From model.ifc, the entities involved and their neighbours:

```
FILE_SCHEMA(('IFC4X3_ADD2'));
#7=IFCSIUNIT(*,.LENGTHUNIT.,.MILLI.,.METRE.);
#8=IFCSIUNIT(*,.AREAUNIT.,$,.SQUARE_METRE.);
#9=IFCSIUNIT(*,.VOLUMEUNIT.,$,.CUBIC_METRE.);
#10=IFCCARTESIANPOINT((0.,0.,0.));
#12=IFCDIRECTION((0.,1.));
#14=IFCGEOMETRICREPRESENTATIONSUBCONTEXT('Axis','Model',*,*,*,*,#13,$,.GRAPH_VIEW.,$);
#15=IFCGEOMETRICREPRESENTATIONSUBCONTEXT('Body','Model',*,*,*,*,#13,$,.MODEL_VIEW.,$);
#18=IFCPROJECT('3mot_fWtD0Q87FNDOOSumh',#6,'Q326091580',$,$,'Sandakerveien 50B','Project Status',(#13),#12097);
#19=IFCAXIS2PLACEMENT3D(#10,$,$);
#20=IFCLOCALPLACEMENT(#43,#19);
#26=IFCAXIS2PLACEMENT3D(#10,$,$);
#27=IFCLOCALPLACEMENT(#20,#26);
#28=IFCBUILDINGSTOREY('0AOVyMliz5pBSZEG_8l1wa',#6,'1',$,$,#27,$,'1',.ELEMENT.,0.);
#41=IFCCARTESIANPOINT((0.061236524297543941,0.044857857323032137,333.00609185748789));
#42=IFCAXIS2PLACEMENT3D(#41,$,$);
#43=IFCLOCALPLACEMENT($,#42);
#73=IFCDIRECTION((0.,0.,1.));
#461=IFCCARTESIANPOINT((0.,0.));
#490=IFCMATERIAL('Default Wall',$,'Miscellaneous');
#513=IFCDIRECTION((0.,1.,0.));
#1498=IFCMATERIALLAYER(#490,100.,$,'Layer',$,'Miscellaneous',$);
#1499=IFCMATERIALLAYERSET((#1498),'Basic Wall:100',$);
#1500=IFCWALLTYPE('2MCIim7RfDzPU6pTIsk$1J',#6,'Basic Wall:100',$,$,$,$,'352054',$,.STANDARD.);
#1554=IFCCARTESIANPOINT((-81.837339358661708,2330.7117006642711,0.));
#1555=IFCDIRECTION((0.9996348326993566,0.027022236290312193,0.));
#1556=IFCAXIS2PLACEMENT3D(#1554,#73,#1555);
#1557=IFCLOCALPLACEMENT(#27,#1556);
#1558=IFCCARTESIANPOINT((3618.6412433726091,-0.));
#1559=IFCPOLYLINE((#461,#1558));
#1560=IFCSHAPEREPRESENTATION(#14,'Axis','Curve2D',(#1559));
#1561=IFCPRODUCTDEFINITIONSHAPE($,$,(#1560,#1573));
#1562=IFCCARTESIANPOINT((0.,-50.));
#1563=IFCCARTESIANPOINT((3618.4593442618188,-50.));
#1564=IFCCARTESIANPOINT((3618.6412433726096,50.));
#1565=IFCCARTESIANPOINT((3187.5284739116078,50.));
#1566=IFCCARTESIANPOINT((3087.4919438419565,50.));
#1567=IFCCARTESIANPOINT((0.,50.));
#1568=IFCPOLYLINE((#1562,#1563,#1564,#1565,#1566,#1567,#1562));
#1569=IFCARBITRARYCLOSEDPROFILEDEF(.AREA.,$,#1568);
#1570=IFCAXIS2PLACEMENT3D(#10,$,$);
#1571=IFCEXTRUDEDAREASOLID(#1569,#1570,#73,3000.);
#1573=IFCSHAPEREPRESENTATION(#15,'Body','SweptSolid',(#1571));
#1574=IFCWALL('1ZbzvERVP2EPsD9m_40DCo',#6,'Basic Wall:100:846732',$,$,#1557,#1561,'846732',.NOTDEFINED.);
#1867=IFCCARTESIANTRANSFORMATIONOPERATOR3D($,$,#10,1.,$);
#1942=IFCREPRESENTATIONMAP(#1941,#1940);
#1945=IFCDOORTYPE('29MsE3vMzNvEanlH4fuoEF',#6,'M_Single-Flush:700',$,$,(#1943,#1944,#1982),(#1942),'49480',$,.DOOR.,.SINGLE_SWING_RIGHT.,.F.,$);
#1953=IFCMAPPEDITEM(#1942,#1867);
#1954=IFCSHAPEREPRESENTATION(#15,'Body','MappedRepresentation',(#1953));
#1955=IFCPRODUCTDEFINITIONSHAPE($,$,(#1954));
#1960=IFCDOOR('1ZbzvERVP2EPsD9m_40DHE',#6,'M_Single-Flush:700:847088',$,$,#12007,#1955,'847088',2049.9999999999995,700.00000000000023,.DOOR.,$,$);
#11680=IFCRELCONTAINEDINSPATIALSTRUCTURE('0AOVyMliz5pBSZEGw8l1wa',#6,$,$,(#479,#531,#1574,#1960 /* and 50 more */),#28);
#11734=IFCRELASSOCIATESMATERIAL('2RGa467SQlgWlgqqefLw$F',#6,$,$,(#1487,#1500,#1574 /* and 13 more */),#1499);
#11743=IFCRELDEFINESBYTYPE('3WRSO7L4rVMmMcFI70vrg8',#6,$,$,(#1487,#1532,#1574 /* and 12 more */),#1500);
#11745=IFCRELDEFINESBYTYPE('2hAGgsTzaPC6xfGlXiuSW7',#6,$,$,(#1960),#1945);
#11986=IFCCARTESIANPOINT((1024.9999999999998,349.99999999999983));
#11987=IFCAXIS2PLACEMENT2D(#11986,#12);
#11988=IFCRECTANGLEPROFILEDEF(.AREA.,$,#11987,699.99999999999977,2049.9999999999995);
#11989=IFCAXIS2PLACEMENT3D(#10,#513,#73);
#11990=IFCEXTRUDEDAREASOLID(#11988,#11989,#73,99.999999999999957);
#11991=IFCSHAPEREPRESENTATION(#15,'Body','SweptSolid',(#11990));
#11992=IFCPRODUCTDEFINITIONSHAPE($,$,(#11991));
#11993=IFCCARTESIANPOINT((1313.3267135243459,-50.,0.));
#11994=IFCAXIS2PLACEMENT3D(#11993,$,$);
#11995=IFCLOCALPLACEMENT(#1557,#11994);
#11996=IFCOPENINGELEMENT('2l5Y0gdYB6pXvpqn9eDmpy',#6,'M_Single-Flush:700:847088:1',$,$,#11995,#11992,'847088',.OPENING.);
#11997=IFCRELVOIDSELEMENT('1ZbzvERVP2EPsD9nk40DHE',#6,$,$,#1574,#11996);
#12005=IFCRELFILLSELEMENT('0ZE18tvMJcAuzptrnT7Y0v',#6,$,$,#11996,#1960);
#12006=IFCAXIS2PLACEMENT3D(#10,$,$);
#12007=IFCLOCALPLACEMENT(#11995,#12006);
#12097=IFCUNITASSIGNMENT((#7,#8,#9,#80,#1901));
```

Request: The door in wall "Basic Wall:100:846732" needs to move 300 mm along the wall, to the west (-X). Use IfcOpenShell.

```python
import ifcopenshell
import ifcopenshell.api.geometry
import ifcopenshell.util.placement

model = ifcopenshell.open("model.ifc")

door = model.by_id(1960)
opening = door.FillsVoids[0].RelatingOpeningElement
wall = opening.VoidsElements[0].RelatingBuildingElement

wall_matrix = ifcopenshell.util.placement.get_local_placement(wall.ObjectPlacement)
shift = wall_matrix[:3, 0] * -300.0
before = ifcopenshell.util.placement.get_local_placement(door.ObjectPlacement)[:3, 3].copy()

# The door is placed relative to its opening, so it follows when the opening moves.
matrix = ifcopenshell.util.placement.get_local_placement(opening.ObjectPlacement)
matrix[:3, 3] += shift
ifcopenshell.api.geometry.edit_object_placement(
    model, product=opening, matrix=matrix, is_si=False, should_transform_children=True
)

after = ifcopenshell.util.placement.get_local_placement(door.ObjectPlacement)[:3, 3]
print("door moved by", (after - before).round(3) + 0.0)

model.write("model_edited.ifc")
```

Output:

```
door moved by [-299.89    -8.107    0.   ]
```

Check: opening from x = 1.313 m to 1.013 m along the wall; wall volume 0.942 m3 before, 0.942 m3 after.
